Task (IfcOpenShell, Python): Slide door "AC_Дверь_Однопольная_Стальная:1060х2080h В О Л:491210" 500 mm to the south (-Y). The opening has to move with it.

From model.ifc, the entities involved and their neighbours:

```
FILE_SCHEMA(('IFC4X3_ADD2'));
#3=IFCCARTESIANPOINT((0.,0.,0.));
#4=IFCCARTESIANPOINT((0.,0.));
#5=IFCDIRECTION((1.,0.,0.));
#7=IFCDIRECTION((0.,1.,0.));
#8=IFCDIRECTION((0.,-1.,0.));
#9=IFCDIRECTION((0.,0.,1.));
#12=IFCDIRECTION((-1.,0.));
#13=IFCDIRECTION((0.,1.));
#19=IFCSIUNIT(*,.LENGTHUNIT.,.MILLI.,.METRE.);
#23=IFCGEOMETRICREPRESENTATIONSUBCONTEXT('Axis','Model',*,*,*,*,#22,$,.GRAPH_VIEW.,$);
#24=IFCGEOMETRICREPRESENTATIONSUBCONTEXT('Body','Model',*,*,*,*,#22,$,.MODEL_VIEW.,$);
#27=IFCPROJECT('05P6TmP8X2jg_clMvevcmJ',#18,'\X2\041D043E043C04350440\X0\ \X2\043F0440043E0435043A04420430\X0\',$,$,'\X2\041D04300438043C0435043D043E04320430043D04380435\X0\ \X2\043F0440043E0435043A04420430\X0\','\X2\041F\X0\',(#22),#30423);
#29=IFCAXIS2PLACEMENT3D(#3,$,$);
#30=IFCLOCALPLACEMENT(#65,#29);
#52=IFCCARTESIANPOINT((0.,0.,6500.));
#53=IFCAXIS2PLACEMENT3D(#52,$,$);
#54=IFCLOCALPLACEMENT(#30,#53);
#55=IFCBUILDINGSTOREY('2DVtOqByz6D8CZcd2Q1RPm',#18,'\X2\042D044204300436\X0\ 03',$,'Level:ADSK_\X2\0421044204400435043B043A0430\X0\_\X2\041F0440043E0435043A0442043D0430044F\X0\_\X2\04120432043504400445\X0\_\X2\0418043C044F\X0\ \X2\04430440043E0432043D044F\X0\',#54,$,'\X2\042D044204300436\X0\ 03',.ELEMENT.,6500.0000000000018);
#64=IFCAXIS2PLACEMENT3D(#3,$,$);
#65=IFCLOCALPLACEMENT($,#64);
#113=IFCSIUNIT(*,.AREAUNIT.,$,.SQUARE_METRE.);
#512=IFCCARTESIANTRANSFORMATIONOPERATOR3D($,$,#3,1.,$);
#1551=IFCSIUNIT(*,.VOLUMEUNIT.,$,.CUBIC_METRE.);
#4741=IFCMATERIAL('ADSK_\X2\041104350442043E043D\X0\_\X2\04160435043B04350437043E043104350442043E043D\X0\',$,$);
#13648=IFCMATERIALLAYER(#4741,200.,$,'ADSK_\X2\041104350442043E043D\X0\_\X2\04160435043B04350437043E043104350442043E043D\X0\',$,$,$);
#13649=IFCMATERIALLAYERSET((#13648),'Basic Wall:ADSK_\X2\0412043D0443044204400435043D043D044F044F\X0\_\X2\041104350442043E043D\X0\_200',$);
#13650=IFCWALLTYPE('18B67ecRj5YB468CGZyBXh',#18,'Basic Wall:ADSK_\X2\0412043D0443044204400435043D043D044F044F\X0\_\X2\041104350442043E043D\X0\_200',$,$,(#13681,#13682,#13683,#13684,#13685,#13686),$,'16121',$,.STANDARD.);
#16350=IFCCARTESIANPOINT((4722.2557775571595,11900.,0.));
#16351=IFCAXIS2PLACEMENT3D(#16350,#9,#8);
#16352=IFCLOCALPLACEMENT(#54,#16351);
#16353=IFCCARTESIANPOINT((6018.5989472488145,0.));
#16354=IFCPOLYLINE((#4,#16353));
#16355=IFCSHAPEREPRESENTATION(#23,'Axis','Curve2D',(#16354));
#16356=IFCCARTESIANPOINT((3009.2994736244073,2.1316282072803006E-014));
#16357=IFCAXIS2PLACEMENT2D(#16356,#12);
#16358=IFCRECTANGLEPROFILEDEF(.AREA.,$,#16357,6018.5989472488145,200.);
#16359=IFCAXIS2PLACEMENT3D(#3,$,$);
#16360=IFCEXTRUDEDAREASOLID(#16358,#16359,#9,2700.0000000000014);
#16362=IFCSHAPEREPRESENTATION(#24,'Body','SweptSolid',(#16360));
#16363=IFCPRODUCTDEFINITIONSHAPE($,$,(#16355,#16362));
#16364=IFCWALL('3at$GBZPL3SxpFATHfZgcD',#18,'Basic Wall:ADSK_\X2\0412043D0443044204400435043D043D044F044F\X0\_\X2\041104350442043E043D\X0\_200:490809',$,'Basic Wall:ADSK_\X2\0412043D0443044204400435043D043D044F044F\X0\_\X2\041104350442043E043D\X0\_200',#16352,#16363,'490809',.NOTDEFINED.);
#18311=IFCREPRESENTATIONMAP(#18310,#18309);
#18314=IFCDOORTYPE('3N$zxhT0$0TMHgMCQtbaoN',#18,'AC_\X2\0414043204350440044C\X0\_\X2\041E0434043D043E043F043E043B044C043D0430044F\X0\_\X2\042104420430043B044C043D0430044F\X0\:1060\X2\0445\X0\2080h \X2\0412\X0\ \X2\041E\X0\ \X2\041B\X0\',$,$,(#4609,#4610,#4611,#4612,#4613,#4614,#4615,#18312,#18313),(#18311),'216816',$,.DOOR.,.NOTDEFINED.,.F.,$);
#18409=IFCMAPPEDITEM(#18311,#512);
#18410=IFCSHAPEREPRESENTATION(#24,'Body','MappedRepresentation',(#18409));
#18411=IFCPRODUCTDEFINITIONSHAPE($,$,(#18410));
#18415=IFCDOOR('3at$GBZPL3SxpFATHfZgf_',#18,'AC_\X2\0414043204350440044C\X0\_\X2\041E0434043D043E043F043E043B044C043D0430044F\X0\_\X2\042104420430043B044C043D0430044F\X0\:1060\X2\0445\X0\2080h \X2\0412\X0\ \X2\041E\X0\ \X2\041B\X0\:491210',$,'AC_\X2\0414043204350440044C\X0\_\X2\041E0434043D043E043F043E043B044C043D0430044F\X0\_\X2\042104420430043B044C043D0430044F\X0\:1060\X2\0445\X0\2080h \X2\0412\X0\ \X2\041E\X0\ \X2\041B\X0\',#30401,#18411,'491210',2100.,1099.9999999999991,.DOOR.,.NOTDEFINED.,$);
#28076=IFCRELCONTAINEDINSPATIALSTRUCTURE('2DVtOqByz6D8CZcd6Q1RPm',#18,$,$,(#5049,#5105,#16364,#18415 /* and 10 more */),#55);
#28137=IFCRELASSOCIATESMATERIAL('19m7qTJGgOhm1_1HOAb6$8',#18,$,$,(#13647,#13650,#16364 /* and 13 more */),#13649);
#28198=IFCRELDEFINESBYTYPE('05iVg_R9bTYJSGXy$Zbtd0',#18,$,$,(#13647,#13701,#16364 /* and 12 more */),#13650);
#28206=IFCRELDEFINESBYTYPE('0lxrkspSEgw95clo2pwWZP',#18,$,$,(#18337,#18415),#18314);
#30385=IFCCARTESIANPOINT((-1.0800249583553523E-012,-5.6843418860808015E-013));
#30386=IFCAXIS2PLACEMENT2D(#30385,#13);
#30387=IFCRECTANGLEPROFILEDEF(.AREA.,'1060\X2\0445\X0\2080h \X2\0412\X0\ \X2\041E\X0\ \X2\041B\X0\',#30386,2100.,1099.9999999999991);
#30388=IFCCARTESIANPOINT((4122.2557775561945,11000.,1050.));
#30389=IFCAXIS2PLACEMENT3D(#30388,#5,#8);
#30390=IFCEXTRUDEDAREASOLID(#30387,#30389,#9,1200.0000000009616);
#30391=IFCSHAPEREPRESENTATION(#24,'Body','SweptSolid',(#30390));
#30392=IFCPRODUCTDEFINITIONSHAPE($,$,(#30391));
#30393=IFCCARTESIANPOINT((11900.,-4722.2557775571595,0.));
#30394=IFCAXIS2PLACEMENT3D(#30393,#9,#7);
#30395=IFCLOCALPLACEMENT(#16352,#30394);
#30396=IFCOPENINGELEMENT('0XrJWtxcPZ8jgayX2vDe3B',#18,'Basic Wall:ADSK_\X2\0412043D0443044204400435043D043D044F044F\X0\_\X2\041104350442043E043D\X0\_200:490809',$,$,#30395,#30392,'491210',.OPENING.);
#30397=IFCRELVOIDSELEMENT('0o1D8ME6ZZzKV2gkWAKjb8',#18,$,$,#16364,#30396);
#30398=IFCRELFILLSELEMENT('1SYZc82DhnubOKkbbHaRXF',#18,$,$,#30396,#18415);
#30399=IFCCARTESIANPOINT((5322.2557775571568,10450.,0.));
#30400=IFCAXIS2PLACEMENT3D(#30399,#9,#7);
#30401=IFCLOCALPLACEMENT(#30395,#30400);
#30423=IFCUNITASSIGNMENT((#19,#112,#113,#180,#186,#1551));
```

```python
import ifcopenshell
import ifcopenshell.api.geometry
import ifcopenshell.util.placement

model = ifcopenshell.open("model.ifc")

door = model.by_id(18415)
opening = door.FillsVoids[0].RelatingOpeningElement
wall = opening.VoidsElements[0].RelatingBuildingElement

wall_matrix = ifcopenshell.util.placement.get_local_placement(wall.ObjectPlacement)
shift = wall_matrix[:3, 0] * 500.0
before = ifcopenshell.util.placement.get_local_placement(door.ObjectPlacement)[:3, 3].copy()

# The door is placed relative to its opening, so it follows when the opening moves.
matrix = ifcopenshell.util.placement.get_local_placement(opening.ObjectPlacement)
matrix[:3, 3] += shift
ifcopenshell.api.geometry.edit_object_placement(
    model, product=opening, matrix=matrix, is_si=False, should_transform_children=True
)

after = ifcopenshell.util.placement.get_local_placement(door.ObjectPlacement)[:3, 3]
print("door moved by", (after - before).round(3) + 0.0)

model.write("model_v2.ifc")
```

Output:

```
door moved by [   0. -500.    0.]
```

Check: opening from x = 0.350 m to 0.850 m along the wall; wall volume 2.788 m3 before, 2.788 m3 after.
